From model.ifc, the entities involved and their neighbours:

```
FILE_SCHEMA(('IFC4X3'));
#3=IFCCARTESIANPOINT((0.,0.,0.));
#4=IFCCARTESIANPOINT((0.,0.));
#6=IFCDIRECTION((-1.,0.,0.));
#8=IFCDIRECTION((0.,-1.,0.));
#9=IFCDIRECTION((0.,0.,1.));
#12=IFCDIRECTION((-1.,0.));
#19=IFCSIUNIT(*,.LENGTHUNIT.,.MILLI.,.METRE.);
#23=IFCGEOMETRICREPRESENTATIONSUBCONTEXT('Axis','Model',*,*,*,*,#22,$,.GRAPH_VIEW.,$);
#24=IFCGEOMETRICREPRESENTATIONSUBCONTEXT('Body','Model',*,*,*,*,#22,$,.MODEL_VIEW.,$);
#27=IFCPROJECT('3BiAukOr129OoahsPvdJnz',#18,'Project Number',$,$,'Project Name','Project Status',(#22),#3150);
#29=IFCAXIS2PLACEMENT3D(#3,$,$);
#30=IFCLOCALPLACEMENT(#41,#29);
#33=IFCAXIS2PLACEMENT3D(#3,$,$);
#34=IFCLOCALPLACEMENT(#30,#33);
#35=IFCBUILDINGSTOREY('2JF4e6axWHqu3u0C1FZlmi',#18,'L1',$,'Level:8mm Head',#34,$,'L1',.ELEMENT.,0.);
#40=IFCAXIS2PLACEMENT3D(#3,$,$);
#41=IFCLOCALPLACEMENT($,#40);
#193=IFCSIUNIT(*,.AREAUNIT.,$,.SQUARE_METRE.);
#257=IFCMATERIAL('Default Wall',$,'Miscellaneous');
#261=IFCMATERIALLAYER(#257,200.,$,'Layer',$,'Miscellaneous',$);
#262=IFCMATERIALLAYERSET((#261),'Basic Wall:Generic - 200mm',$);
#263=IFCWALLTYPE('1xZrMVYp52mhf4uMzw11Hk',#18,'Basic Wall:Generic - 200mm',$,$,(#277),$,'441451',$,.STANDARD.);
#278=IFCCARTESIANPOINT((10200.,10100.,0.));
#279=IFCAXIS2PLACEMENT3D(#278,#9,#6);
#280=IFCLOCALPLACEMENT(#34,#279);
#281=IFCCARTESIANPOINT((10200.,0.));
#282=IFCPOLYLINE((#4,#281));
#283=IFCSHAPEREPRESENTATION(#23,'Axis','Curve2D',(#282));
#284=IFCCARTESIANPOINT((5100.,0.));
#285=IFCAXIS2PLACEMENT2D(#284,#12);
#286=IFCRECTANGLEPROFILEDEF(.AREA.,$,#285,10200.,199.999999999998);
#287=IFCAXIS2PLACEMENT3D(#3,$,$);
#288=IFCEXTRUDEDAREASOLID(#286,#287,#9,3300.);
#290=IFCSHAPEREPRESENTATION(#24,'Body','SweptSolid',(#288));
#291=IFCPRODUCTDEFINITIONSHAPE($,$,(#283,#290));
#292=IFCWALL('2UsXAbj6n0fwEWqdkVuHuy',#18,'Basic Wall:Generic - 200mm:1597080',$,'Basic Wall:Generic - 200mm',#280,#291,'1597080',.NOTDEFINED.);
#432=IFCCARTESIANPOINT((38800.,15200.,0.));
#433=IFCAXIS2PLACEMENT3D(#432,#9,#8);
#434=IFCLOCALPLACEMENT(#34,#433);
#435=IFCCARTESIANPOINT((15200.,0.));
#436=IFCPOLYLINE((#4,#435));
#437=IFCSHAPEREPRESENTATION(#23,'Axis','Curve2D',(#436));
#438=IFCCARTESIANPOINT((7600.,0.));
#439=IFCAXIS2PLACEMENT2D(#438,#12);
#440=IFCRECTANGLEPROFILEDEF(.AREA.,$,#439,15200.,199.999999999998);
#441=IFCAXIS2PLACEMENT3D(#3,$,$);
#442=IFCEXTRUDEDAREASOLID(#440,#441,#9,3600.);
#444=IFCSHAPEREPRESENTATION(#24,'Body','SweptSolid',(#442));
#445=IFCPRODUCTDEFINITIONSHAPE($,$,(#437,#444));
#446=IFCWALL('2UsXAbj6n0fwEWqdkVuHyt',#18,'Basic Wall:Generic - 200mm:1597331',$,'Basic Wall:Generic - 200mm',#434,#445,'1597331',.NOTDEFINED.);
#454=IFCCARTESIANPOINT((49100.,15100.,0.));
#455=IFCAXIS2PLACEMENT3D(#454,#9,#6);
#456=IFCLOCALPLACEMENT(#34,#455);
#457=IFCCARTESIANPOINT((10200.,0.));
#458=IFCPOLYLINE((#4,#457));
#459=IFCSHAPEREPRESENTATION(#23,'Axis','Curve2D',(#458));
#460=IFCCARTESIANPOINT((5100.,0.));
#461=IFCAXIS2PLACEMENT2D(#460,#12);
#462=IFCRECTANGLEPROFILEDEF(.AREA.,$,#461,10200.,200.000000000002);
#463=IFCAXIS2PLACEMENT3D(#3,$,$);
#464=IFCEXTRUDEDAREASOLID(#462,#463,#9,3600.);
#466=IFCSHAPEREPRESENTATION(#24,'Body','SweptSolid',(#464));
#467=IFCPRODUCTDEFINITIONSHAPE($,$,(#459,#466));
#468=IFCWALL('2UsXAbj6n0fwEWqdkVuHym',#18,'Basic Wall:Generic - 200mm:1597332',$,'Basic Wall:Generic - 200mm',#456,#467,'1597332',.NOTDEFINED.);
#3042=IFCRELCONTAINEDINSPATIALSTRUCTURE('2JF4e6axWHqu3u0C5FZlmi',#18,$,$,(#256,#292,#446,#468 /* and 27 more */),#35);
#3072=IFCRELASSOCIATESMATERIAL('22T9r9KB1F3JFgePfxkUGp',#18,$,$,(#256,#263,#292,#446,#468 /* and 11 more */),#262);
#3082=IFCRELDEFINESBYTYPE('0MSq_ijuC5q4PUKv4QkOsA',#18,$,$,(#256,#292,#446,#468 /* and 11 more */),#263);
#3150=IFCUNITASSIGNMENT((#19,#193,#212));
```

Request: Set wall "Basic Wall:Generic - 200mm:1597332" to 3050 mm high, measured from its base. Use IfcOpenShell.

```python
import ifcopenshell
import ifcopenshell.geom
import ifcopenshell.util.representation
import ifcopenshell.util.shape
import ifcopenshell.util.unit

model = ifcopenshell.open("model.ifc")
unit_scale = ifcopenshell.util.unit.calculate_unit_scale(model)
settings = ifcopenshell.geom.settings()


def volume(element):
    """Net volume in cubic metres, openings subtracted."""
    shape = ifcopenshell.geom.create_shape(settings, element)
    return ifcopenshell.util.shape.get_volume(shape.geometry)


wall = model.by_id(468)
before = volume(wall)

body = ifcopenshell.util.representation.get_representation(wall, "Model", "Body")
solid = body.Items[0]
old_height = solid.Depth
solid.Depth = 3.05 / unit_scale
after = volume(wall)

print(f"height {old_height:g} -> {solid.Depth:g}, volume {before:.3f} -> {after:.3f} m3")

model.write("model-out.ifc")
```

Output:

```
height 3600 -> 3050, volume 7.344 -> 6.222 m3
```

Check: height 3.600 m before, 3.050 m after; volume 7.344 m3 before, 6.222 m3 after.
